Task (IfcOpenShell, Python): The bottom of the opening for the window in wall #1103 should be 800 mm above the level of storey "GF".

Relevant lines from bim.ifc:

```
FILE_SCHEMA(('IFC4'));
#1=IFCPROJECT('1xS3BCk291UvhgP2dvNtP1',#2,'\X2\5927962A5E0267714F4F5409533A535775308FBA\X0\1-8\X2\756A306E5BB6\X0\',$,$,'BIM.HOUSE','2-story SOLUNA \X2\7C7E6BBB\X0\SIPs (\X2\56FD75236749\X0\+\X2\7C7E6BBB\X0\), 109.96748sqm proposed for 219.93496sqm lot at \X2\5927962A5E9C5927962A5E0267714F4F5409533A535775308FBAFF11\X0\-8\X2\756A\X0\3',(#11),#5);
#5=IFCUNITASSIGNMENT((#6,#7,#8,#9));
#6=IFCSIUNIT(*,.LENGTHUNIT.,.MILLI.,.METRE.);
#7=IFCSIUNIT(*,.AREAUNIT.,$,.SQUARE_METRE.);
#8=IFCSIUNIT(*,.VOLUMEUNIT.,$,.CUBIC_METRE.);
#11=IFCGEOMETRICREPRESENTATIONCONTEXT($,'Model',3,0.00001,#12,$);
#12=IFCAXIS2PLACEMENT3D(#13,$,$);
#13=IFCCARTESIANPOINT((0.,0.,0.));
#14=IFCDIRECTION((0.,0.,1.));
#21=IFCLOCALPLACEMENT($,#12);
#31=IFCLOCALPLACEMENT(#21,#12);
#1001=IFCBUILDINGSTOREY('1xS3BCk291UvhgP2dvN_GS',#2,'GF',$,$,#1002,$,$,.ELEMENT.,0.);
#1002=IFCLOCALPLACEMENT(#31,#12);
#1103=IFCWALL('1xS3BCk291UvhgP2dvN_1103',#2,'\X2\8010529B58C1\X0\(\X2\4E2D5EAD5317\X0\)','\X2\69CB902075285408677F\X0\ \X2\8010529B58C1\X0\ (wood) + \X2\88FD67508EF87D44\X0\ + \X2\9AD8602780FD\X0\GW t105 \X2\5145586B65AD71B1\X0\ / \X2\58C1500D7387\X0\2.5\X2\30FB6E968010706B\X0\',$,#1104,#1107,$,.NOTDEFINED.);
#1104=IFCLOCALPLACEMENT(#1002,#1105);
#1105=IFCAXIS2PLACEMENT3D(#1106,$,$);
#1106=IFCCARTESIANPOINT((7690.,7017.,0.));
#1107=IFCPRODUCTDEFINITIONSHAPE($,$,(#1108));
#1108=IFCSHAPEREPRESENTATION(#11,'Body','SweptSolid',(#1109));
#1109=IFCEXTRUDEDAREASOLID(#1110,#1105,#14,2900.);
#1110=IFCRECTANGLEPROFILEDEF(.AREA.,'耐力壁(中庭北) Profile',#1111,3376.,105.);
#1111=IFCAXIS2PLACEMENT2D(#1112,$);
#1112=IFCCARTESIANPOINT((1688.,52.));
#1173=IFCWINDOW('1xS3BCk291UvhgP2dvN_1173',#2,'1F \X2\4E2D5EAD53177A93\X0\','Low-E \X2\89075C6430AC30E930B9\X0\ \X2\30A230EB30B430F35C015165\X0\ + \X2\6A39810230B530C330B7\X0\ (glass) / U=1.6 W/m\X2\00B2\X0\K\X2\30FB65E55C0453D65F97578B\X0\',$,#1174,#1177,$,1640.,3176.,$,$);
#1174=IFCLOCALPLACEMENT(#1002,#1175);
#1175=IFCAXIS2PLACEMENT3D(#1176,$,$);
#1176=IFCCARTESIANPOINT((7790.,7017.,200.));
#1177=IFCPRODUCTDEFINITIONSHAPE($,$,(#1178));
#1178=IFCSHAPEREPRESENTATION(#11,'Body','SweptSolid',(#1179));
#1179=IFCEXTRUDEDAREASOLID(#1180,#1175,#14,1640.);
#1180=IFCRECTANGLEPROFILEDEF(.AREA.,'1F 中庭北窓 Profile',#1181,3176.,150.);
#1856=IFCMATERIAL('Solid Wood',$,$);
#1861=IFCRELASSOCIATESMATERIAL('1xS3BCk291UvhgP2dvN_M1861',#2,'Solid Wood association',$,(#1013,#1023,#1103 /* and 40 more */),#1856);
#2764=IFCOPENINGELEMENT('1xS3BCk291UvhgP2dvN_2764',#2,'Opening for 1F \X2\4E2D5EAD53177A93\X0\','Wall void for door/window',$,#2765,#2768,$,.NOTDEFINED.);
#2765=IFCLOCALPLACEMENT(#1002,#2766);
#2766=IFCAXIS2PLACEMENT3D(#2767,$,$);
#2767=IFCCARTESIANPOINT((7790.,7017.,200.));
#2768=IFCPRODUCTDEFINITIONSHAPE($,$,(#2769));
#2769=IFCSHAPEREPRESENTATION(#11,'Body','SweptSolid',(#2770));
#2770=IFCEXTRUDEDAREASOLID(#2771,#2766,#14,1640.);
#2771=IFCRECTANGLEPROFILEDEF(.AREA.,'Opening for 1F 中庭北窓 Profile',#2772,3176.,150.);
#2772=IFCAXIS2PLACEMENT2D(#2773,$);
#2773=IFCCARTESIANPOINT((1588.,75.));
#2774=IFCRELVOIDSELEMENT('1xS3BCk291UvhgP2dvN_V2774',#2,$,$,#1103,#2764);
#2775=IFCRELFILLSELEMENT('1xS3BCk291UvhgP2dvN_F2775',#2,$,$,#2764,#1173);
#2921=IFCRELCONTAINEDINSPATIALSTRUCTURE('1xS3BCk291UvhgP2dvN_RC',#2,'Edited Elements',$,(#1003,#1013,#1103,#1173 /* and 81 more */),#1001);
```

```python
import numpy as np
import ifcopenshell
import ifcopenshell.api.geometry
import ifcopenshell.geom
import ifcopenshell.util.element
import ifcopenshell.util.placement
import ifcopenshell.util.shape
import ifcopenshell.util.unit

model = ifcopenshell.open("bim.ifc")
unit_scale = ifcopenshell.util.unit.calculate_unit_scale(model)

window = model.by_guid("1xS3BCk291UvhgP2dvN_1173")
opening = window.FillsVoids[0].RelatingOpeningElement
storey = ifcopenshell.util.element.get_container(window, ifc_class="IfcBuildingStorey")
level = ifcopenshell.util.placement.get_local_placement(storey.ObjectPlacement)[2, 3]

# The opening's origin need not be at the sill, so measure its lowest point.
shape = ifcopenshell.geom.create_shape(ifcopenshell.geom.settings(), opening)
bottom = ifcopenshell.util.shape.get_shape_bottom_elevation(shape, shape.geometry) / unit_scale
dz = level + 800.0 - bottom

shift = np.array([0.0, 0.0, dz])
# The window is not placed relative to its opening, so move both.
for product in (opening, window):
    matrix = ifcopenshell.util.placement.get_local_placement(product.ObjectPlacement)
    matrix[:3, 3] += shift
    ifcopenshell.api.geometry.edit_object_placement(model, product=product, matrix=matrix, is_si=False)

print(f"moved by {dz * unit_scale:+.3f} m")

model.write("bim_updated.ifc")
```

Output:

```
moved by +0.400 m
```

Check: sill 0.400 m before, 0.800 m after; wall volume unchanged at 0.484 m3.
